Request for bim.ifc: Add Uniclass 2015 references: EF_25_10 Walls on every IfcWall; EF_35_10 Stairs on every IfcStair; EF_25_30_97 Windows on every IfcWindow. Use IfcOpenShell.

First a look at what the model holds.

```python
import ifcopenshell

model = ifcopenshell.open("bim.ifc")
print(model.schema)
print("classifications:", [c.Name for c in model.by_type("IfcClassification")])
for ifc_class in ("IfcDoor", "IfcRoof", "IfcStair", "IfcWall", "IfcWindow"):
    print(ifc_class, len(model.by_type(ifc_class)))
```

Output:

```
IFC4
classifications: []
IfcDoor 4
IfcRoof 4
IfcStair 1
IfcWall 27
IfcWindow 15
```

```python
import ifcopenshell
import ifcopenshell.api.classification

model = ifcopenshell.open("bim.ifc")

system = ifcopenshell.api.classification.add_classification(model, classification="Uniclass 2015")

codes = {
    "IfcWall": ("EF_25_10", "Walls"),
    "IfcStair": ("EF_35_10", "Stairs"),
    "IfcWindow": ("EF_25_30_97", "Windows"),
}
for ifc_class, (code, name) in codes.items():
    products = model.by_type(ifc_class)
    ifcopenshell.api.classification.add_reference(
        model, products=products, classification=system, identification=code, name=name
    )
    print(code, len(products))

model.write("bim_v2.ifc")
```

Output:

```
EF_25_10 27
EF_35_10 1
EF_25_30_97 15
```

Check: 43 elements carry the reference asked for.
